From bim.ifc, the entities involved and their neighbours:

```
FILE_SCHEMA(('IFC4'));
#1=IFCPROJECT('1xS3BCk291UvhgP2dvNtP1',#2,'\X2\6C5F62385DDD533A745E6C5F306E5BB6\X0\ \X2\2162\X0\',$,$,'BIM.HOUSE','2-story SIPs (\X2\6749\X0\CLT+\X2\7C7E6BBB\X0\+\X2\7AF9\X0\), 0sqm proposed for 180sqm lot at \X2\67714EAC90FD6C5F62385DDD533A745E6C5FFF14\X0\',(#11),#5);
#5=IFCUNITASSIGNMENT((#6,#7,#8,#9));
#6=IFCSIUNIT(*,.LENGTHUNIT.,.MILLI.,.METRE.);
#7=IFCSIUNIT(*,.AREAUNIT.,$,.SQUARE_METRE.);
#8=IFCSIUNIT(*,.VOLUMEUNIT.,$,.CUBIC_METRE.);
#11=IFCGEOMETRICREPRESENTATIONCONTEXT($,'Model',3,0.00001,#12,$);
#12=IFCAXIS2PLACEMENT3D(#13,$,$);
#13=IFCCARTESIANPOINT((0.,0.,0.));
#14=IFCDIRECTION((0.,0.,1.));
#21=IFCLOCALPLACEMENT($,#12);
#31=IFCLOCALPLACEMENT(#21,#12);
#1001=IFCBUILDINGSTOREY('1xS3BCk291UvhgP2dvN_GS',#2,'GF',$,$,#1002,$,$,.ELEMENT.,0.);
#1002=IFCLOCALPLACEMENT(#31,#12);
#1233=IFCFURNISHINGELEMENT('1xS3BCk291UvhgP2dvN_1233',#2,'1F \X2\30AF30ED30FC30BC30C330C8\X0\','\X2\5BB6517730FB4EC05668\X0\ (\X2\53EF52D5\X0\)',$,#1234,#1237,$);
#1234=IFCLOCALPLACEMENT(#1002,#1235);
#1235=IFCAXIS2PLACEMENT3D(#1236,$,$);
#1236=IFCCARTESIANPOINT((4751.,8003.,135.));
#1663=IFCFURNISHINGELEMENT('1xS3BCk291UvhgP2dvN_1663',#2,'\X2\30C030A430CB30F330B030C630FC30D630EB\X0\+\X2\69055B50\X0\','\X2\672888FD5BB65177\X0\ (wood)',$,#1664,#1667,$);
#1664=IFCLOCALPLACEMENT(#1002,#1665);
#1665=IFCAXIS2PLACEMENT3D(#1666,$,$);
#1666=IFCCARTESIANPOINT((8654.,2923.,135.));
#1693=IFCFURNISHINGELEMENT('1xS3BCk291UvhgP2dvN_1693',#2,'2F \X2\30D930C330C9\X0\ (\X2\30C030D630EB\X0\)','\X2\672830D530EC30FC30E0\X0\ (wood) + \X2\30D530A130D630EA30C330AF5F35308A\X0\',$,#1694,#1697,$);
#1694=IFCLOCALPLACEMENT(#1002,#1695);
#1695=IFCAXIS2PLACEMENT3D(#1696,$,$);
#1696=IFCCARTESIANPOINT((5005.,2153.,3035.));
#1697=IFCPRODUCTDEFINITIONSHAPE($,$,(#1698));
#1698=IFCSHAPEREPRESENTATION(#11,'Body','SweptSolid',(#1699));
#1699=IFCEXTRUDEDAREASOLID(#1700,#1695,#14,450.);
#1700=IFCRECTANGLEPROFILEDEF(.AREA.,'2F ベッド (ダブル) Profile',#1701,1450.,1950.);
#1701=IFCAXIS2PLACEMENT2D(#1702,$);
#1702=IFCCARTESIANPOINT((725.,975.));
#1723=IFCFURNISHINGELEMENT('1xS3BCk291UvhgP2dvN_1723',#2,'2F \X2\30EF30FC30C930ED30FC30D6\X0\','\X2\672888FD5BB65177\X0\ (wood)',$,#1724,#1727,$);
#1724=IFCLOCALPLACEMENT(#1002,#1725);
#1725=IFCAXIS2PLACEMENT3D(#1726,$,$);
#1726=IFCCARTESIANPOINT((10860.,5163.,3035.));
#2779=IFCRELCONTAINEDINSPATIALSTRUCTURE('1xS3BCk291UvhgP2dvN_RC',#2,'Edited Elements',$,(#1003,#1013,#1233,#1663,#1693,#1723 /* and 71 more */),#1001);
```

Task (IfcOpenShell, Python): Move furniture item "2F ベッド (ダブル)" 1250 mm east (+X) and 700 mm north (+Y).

```python
import ifcopenshell
import ifcopenshell.api.geometry
import ifcopenshell.util.placement

model = ifcopenshell.open("bim.ifc")

item = model.by_guid("1xS3BCk291UvhgP2dvN_1693")
matrix = ifcopenshell.util.placement.get_local_placement(item.ObjectPlacement)
matrix[0, 3] += 1250.0
matrix[1, 3] += 700.0
ifcopenshell.api.geometry.edit_object_placement(model, product=item, matrix=matrix, is_si=False)

print(ifcopenshell.util.placement.get_local_placement(item.ObjectPlacement).round(3) + 0.0)

model.write("bim_v2.ifc")
```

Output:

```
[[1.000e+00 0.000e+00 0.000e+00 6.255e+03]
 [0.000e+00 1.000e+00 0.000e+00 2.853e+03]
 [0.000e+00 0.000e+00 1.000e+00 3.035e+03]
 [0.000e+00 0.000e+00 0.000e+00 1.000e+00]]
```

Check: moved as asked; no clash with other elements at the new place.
